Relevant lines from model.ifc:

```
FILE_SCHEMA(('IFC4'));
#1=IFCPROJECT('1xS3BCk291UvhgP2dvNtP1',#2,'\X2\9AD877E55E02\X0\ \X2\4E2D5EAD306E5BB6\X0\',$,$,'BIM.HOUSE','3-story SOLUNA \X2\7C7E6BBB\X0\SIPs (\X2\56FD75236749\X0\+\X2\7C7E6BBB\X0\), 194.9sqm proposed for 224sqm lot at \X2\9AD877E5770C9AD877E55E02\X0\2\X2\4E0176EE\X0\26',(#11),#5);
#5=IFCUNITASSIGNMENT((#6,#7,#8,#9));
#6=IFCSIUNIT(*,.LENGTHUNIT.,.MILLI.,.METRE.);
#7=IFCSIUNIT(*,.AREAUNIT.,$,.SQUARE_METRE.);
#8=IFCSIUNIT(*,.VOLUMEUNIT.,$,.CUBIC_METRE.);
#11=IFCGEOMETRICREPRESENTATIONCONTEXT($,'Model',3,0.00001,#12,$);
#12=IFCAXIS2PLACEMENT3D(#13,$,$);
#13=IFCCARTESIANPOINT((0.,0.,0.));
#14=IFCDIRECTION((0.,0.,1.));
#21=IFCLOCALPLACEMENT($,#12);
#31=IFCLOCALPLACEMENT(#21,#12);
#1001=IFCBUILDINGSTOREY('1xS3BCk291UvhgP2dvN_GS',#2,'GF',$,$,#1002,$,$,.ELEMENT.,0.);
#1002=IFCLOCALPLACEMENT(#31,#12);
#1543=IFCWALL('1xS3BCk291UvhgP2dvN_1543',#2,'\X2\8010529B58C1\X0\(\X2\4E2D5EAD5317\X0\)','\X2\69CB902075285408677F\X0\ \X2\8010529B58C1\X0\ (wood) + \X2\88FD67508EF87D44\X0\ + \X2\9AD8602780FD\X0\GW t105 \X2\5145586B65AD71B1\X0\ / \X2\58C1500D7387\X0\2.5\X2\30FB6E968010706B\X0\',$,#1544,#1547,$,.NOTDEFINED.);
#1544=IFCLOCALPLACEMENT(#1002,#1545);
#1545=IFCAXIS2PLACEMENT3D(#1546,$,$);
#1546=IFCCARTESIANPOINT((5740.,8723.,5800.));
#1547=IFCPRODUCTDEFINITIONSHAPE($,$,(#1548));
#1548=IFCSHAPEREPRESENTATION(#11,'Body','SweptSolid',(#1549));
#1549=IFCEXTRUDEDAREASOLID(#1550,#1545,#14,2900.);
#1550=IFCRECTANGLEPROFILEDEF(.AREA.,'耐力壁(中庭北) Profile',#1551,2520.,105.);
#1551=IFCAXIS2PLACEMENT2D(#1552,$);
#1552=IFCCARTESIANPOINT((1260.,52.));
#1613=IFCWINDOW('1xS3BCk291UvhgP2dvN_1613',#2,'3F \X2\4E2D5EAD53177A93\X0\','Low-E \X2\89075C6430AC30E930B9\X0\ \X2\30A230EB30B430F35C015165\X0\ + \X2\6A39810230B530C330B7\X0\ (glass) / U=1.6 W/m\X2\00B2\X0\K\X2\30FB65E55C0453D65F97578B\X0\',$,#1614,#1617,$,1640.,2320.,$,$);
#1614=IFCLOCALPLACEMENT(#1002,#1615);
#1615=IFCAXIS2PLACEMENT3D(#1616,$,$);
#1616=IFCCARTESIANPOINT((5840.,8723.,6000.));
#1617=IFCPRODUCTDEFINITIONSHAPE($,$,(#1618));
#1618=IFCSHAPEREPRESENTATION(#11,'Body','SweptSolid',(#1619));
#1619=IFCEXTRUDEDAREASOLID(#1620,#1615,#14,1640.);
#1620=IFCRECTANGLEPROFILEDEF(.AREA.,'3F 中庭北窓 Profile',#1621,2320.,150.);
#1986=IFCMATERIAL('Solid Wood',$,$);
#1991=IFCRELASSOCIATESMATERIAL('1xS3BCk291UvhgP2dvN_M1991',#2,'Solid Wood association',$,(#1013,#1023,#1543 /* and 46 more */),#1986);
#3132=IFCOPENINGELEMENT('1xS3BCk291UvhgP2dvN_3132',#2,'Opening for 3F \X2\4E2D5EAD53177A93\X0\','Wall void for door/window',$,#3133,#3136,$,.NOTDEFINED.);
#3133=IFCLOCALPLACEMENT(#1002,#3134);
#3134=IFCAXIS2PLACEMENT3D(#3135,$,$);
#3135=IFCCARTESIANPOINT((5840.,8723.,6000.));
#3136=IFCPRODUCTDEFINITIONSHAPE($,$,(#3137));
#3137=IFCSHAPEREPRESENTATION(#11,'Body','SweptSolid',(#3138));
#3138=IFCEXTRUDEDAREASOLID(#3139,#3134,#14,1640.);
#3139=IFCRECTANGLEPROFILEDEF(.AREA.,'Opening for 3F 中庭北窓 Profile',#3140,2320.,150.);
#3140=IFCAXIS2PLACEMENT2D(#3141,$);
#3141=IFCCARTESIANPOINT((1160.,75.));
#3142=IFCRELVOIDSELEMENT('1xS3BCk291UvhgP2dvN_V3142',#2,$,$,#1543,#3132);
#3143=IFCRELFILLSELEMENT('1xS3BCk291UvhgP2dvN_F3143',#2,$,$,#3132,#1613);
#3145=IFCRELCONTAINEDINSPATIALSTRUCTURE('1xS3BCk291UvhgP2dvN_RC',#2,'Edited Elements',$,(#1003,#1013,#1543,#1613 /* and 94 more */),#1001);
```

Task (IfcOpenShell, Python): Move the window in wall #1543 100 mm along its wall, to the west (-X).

```python
import ifcopenshell
import ifcopenshell.api.geometry
import ifcopenshell.util.placement
import ifcopenshell.util.unit

model = ifcopenshell.open("model.ifc")
unit_scale = ifcopenshell.util.unit.calculate_unit_scale(model)

window = model.by_guid("1xS3BCk291UvhgP2dvN_1613")
opening = window.FillsVoids[0].RelatingOpeningElement
wall = opening.VoidsElements[0].RelatingBuildingElement

wall_matrix = ifcopenshell.util.placement.get_local_placement(wall.ObjectPlacement)
shift = wall_matrix[:3, 0] * -0.1 / unit_scale
before = ifcopenshell.util.placement.get_local_placement(window.ObjectPlacement)[:3, 3].copy()

# The window is not placed relative to its opening, so move both.
for product in (opening, window):
    matrix = ifcopenshell.util.placement.get_local_placement(product.ObjectPlacement)
    matrix[:3, 3] += shift
    ifcopenshell.api.geometry.edit_object_placement(model, product=product, matrix=matrix, is_si=False)

after = ifcopenshell.util.placement.get_local_placement(window.ObjectPlacement)[:3, 3]
print("window moved by", (after - before).round(3) + 0.0)

model.write("model_edited.ifc")
```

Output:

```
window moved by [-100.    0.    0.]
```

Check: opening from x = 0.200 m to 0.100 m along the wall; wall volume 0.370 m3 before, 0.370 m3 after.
